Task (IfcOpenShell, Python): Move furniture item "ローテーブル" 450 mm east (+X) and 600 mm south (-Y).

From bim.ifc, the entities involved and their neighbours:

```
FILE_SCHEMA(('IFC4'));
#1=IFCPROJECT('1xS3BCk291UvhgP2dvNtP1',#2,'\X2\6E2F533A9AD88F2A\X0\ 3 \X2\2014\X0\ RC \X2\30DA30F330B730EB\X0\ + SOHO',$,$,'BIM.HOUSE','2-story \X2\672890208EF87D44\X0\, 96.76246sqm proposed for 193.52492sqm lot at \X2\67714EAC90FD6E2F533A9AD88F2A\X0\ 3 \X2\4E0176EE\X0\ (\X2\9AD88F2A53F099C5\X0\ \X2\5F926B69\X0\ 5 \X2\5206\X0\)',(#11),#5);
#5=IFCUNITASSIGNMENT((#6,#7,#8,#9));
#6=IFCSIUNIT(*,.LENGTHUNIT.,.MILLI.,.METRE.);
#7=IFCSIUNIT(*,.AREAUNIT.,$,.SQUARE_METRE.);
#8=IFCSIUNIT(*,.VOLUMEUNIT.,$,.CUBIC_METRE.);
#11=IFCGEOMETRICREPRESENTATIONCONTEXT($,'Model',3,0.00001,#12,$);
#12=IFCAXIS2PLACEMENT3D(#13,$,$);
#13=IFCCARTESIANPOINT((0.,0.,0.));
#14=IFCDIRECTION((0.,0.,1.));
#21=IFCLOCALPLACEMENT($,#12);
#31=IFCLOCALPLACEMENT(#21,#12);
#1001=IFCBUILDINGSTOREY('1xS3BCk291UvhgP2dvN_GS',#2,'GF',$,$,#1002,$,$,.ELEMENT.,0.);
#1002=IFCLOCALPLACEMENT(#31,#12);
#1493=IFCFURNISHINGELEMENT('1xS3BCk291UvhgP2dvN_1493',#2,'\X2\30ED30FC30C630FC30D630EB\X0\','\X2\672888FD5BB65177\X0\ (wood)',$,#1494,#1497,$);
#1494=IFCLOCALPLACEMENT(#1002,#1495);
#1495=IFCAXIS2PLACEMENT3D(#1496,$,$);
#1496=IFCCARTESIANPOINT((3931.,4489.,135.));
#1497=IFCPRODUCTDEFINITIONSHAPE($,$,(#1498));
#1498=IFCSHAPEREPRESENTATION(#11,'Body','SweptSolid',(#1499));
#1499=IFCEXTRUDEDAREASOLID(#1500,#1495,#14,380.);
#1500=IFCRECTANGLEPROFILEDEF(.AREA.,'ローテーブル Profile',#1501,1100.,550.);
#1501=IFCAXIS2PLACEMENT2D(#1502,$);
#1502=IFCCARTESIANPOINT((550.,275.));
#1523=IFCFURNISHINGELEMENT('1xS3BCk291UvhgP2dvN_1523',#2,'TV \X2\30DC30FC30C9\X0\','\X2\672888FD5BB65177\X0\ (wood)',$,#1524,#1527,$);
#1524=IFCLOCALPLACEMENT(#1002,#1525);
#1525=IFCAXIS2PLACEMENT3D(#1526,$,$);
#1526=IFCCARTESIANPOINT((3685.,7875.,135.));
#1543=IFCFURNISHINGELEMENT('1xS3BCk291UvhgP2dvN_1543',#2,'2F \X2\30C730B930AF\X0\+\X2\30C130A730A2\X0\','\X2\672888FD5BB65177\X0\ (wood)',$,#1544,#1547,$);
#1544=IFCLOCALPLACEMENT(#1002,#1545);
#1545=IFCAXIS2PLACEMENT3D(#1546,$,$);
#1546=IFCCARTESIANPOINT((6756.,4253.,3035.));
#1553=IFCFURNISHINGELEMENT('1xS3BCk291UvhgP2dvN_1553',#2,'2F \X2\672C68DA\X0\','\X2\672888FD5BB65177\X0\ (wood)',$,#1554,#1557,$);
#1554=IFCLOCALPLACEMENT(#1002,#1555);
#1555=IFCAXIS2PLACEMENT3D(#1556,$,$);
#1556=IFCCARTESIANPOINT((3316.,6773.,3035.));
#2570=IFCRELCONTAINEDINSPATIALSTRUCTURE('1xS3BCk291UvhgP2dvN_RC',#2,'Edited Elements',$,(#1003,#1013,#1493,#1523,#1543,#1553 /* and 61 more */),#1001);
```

```python
import ifcopenshell
import ifcopenshell.api.geometry
import ifcopenshell.util.placement
import ifcopenshell.util.unit

model = ifcopenshell.open("bim.ifc")
unit_scale = ifcopenshell.util.unit.calculate_unit_scale(model)

item = model.by_guid("1xS3BCk291UvhgP2dvN_1493")
matrix = ifcopenshell.util.placement.get_local_placement(item.ObjectPlacement)
matrix[0, 3] += 0.45 / unit_scale
matrix[1, 3] -= 0.6 / unit_scale
ifcopenshell.api.geometry.edit_object_placement(model, product=item, matrix=matrix, is_si=False)

print(ifcopenshell.util.placement.get_local_placement(item.ObjectPlacement).round(3) + 0.0)

model.write("bim_edited.ifc")
```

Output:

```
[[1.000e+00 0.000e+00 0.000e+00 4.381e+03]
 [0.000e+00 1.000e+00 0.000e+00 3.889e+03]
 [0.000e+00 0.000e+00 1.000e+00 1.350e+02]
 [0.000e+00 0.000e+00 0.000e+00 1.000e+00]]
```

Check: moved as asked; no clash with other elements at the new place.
